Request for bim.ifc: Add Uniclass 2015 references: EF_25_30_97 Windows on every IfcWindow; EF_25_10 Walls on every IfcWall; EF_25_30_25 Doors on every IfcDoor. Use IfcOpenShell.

First a look at what the model holds.

```python
import ifcopenshell

model = ifcopenshell.open("bim.ifc")
print(model.schema)
print("classifications:", [c.Name for c in model.by_type("IfcClassification")])
for ifc_class in ("IfcDoor", "IfcRoof", "IfcStair", "IfcWall", "IfcWindow"):
    print(ifc_class, len(model.by_type(ifc_class)))
```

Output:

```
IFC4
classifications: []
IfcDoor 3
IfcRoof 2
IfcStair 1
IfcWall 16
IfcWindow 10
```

```python
import ifcopenshell
import ifcopenshell.api.classification

model = ifcopenshell.open("bim.ifc")

system = ifcopenshell.api.classification.add_classification(model, classification="Uniclass 2015")

codes = {
    "IfcWindow": ("EF_25_30_97", "Windows"),
    "IfcWall": ("EF_25_10", "Walls"),
    "IfcDoor": ("EF_25_30_25", "Doors"),
}
for ifc_class, (code, name) in codes.items():
    products = model.by_type(ifc_class)
    ifcopenshell.api.classification.add_reference(
        model, products=products, classification=system, identification=code, name=name
    )
    print(code, len(products))

model.write("bim-out.ifc")
```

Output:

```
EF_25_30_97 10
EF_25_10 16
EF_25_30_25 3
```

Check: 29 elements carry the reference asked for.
